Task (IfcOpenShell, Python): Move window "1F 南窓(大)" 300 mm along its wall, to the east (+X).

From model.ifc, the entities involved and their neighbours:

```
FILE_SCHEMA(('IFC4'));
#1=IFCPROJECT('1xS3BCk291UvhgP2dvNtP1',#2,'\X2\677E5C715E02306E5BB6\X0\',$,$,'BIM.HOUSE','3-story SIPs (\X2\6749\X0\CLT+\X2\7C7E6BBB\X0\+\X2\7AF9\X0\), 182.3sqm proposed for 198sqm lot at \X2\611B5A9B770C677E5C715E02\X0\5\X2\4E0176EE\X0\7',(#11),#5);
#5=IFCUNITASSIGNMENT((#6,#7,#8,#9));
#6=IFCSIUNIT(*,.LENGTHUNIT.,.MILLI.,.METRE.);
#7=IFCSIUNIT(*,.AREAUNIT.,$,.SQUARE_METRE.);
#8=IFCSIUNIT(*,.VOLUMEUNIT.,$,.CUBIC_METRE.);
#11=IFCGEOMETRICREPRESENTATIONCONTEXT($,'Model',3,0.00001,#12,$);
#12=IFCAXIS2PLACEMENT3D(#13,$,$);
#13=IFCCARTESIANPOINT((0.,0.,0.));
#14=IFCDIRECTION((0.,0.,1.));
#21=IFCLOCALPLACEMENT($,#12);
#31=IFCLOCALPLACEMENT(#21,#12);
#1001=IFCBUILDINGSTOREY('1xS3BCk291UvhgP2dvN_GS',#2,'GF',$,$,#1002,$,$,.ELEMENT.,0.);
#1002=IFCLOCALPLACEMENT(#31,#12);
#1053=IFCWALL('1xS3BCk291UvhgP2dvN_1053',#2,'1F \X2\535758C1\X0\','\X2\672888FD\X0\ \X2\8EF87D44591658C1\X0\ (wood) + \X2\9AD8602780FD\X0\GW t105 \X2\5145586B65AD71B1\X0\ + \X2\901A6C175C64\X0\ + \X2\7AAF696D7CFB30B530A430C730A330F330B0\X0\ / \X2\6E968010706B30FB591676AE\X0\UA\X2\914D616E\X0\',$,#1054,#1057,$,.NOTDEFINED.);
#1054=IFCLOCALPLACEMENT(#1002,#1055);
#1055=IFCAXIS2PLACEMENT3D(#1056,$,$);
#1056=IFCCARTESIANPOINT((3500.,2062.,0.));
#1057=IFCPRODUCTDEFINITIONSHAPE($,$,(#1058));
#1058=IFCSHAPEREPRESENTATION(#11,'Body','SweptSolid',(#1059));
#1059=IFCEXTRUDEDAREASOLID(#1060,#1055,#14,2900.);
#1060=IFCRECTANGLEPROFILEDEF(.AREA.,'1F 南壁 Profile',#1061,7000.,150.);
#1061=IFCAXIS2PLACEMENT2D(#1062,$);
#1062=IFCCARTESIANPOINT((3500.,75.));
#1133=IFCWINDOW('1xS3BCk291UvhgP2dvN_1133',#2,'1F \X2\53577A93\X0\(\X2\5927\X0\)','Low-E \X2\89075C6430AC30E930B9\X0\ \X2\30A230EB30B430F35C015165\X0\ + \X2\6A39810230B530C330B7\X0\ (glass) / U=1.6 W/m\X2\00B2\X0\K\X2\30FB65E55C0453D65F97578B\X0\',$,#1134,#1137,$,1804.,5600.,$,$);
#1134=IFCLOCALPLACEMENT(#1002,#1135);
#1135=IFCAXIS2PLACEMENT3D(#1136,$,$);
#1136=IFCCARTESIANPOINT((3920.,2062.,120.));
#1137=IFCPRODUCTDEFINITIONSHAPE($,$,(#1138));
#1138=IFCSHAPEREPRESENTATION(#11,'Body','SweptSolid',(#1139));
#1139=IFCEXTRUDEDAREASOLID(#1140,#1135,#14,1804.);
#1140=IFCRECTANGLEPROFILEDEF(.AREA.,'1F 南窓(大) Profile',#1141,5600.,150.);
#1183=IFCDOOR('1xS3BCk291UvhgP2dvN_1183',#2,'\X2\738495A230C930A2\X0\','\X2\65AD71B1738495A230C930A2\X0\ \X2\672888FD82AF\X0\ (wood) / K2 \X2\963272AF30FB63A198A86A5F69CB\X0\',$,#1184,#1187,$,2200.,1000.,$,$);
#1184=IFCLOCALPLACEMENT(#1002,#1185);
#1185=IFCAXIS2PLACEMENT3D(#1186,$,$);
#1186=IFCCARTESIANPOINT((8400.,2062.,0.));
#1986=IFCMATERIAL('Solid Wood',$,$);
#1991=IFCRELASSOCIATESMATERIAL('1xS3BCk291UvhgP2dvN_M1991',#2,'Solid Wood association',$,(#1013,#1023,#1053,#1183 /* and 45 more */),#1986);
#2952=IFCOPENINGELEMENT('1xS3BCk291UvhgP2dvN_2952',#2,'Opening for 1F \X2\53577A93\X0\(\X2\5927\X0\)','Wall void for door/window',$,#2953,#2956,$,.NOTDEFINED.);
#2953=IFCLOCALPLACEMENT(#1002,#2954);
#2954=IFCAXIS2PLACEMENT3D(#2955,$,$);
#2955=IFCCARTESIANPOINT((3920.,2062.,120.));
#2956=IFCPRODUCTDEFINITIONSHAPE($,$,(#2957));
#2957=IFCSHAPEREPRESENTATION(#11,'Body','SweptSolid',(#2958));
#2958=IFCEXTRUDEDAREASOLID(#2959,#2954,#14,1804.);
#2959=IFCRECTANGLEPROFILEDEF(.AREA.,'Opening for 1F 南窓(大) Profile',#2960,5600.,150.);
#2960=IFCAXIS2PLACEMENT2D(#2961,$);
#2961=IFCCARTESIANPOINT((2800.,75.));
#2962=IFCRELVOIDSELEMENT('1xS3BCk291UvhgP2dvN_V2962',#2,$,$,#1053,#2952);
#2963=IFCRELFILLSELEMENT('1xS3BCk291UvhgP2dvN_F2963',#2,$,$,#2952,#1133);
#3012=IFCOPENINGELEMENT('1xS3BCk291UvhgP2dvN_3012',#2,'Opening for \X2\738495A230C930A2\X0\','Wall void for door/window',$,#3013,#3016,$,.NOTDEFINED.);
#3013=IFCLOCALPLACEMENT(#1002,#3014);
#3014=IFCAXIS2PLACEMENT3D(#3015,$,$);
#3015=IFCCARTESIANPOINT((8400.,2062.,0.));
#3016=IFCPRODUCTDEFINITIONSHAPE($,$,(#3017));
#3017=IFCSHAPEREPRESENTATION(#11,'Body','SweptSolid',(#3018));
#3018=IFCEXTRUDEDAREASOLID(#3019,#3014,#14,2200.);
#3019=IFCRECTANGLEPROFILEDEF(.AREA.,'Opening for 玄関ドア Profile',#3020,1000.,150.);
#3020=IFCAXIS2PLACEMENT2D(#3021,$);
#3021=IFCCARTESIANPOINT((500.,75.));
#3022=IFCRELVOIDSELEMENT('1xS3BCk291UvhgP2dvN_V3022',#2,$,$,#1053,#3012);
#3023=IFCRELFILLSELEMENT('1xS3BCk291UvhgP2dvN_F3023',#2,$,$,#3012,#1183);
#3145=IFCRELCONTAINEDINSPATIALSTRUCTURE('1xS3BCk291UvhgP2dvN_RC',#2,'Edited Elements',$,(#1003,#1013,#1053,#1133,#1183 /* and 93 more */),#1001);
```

```python
import ifcopenshell
import ifcopenshell.api.geometry
import ifcopenshell.util.placement
import ifcopenshell.util.unit

model = ifcopenshell.open("model.ifc")
unit_scale = ifcopenshell.util.unit.calculate_unit_scale(model)

window = model.by_guid("1xS3BCk291UvhgP2dvN_1133")
opening = window.FillsVoids[0].RelatingOpeningElement
wall = opening.VoidsElements[0].RelatingBuildingElement

wall_matrix = ifcopenshell.util.placement.get_local_placement(wall.ObjectPlacement)
shift = wall_matrix[:3, 0] * 0.3 / unit_scale
before = ifcopenshell.util.placement.get_local_placement(window.ObjectPlacement)[:3, 3].copy()

# The window is not placed relative to its opening, so move both.
for product in (opening, window):
    matrix = ifcopenshell.util.placement.get_local_placement(product.ObjectPlacement)
    matrix[:3, 3] += shift
    ifcopenshell.api.geometry.edit_object_placement(model, product=product, matrix=matrix, is_si=False)

after = ifcopenshell.util.placement.get_local_placement(window.ObjectPlacement)[:3, 3]
print("window moved by", (after - before).round(3) + 0.0)

model.write("model-out.ifc")
```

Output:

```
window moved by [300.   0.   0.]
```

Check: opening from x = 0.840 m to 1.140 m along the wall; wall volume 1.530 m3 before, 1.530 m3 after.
